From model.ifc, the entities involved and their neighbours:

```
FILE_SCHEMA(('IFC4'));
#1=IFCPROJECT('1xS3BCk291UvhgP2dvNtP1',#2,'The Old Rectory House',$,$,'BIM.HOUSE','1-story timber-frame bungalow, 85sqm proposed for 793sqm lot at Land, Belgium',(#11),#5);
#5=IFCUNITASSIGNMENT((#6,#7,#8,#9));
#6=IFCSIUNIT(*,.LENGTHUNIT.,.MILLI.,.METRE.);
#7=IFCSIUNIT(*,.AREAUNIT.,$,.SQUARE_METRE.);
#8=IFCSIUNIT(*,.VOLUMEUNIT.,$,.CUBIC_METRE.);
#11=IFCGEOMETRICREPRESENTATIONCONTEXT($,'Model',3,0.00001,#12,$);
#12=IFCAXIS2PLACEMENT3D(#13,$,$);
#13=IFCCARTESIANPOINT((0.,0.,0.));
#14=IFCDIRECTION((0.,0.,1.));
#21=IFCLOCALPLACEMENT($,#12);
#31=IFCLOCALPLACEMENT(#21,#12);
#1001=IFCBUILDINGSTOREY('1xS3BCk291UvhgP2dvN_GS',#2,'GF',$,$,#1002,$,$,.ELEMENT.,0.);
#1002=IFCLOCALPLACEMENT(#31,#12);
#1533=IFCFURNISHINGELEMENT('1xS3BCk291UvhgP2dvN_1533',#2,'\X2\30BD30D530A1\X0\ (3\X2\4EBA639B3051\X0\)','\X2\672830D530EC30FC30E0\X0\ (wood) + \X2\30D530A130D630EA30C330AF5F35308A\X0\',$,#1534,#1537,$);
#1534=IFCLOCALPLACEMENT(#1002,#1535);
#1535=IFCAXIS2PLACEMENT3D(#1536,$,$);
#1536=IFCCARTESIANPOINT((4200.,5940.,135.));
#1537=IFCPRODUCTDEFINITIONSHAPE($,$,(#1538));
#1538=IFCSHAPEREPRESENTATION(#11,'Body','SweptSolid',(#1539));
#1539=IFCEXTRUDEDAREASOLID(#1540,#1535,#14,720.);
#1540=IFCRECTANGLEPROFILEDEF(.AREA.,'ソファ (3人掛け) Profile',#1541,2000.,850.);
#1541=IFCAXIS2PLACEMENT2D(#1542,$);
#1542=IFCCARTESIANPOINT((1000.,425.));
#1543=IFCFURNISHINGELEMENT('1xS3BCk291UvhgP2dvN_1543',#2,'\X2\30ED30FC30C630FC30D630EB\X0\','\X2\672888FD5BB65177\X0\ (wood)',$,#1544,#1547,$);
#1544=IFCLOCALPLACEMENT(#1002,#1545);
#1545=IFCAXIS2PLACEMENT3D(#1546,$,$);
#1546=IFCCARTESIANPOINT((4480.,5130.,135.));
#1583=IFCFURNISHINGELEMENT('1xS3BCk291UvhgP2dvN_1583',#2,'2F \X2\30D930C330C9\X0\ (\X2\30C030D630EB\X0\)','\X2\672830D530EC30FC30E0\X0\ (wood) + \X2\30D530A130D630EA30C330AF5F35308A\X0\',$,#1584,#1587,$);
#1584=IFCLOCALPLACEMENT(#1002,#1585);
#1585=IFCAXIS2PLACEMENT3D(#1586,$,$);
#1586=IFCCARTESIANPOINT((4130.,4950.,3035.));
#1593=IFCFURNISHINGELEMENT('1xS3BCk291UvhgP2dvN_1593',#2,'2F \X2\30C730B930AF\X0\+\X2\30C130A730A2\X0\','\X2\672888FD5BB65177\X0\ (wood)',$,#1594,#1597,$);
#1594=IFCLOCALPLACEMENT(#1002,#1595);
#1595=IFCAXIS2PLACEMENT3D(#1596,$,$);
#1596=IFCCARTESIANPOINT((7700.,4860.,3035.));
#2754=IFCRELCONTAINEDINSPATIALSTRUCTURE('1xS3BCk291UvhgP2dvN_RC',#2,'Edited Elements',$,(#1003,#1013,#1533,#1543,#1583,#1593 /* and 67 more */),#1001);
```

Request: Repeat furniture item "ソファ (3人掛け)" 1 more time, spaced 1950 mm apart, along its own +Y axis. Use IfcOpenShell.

```python
import ifcopenshell
import ifcopenshell.api.geometry
import ifcopenshell.api.root
import ifcopenshell.util.element
import ifcopenshell.util.placement
import ifcopenshell.util.unit

model = ifcopenshell.open("model.ifc")
unit_scale = ifcopenshell.util.unit.calculate_unit_scale(model)


def reuse_history(source, copy):
    """copy_class also copies each property set's owner history, people and application; keep the originals."""
    for rel in copy.IsDefinedBy:
        if rel.is_a("IfcRelDefinesByProperties") and (history := rel.RelatingPropertyDefinition.OwnerHistory):
            rel.RelatingPropertyDefinition.OwnerHistory = source.OwnerHistory
            ifcopenshell.util.element.remove_deep2(model, history)


source = model.by_guid("1xS3BCk291UvhgP2dvN_1533")
base = ifcopenshell.util.placement.get_local_placement(source.ObjectPlacement)
step = base[:3, 1] * 1.95 / unit_scale

for i in range(1, 2):
    copy = ifcopenshell.api.root.copy_class(model, product=source)
    copy.Representation = ifcopenshell.util.element.copy_deep(
        model, source.Representation, exclude=["IfcGeometricRepresentationContext", "IfcRepresentationMap"]
    )
    reuse_history(source, copy)
    matrix = base.copy()
    matrix[:3, 3] += i * step
    print("added at", matrix[:3, 3].round(3) + 0.0)
    ifcopenshell.api.geometry.edit_object_placement(model, product=copy, matrix=matrix, is_si=False)

model.write("model_updated.ifc")
```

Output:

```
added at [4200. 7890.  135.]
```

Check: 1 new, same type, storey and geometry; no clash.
